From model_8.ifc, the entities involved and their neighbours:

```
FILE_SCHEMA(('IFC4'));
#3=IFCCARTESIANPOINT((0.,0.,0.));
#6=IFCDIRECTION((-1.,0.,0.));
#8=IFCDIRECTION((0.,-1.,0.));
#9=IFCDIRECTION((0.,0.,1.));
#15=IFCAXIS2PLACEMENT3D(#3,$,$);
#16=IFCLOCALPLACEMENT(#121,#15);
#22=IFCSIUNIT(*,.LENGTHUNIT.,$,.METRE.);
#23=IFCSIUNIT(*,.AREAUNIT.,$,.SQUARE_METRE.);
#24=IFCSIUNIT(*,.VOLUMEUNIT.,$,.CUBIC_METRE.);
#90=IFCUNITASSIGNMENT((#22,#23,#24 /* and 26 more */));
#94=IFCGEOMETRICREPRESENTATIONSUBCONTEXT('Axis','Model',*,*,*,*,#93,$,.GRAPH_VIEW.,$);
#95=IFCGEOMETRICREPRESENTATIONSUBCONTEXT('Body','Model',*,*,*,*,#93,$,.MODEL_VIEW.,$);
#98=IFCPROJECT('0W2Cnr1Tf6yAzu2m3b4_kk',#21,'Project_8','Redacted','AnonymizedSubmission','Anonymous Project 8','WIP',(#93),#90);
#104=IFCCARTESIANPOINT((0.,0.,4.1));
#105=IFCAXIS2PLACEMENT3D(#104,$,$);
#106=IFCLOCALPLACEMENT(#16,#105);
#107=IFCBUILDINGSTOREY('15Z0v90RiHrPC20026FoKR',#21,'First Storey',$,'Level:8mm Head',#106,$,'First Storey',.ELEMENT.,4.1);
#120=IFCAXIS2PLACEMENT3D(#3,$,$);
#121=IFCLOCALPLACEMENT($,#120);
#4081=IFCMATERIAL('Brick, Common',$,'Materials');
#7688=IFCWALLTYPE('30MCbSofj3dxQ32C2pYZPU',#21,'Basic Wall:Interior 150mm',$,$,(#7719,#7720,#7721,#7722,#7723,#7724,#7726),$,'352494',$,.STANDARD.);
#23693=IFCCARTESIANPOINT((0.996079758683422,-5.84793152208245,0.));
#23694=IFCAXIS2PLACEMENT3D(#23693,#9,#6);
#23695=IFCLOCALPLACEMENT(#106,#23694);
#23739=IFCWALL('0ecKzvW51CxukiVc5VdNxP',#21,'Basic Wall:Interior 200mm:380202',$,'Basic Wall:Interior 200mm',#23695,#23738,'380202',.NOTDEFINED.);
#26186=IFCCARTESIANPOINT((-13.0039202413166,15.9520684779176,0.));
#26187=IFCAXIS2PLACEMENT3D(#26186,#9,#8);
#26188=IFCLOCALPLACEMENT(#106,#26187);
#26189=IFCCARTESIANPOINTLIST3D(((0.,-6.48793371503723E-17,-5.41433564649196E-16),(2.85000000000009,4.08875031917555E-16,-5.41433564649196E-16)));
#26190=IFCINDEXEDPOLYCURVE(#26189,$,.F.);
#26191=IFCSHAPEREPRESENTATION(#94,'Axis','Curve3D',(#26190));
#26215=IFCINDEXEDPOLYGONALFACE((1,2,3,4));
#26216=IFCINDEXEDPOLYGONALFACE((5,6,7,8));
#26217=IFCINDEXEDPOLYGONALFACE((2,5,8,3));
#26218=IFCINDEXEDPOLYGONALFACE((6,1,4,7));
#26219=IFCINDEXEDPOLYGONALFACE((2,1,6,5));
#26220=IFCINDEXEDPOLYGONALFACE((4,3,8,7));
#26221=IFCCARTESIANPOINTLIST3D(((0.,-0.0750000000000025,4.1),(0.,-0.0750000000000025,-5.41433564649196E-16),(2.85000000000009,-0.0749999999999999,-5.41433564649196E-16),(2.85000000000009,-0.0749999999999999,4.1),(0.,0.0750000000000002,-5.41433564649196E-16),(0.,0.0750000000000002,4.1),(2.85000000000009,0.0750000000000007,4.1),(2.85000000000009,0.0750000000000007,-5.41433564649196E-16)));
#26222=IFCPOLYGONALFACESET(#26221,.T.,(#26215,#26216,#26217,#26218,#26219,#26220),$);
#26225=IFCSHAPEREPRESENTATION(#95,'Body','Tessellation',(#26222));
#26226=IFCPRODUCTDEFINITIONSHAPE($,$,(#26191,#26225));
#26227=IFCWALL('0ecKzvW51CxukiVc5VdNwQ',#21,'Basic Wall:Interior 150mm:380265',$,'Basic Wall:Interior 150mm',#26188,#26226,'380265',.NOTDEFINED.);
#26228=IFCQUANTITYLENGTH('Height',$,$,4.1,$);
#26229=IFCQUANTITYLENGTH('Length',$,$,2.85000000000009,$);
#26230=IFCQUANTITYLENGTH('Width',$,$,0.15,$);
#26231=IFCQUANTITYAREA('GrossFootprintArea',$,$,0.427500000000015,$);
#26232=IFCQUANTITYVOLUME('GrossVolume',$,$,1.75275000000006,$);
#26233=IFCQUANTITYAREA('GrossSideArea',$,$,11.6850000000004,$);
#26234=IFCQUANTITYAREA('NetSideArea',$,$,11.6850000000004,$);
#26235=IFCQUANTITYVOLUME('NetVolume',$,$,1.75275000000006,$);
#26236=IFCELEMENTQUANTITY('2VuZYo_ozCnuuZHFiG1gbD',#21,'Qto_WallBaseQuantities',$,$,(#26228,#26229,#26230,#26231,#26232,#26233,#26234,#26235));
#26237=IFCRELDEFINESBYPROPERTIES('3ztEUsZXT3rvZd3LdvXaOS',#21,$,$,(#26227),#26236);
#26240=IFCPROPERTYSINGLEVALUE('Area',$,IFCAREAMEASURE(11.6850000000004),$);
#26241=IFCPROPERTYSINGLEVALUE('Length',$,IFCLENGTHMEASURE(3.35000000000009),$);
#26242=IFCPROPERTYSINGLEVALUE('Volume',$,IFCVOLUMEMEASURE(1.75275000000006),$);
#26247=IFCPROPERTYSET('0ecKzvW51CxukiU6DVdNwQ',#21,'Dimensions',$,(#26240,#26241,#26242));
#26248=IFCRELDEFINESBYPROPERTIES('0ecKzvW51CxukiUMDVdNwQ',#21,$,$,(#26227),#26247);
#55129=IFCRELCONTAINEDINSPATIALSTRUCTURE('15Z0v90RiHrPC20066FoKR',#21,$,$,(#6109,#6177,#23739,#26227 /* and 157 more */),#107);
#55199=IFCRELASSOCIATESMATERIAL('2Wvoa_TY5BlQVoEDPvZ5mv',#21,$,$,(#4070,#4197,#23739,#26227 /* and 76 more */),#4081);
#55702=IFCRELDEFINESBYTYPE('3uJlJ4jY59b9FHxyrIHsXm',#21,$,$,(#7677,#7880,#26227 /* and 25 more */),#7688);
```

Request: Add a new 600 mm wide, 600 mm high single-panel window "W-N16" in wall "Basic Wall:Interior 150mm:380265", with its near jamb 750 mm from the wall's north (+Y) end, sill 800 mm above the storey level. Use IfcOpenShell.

```python
import numpy as np
import ifcopenshell
import ifcopenshell.api.feature
import ifcopenshell.api.geometry
import ifcopenshell.api.pset
import ifcopenshell.api.root
import ifcopenshell.api.spatial
import ifcopenshell.geom
import ifcopenshell.util.element
import ifcopenshell.util.placement
import ifcopenshell.util.representation
import ifcopenshell.util.shape
import ifcopenshell.util.unit

model = ifcopenshell.open("model_8.ifc")
unit_scale = ifcopenshell.util.unit.calculate_unit_scale(model)
area_scale = ifcopenshell.util.unit.calculate_unit_scale(model, "AREAUNIT")
volume_scale = ifcopenshell.util.unit.calculate_unit_scale(model, "VOLUMEUNIT")
settings = ifcopenshell.geom.settings()


def volume(element):
    """Net volume in cubic metres, openings subtracted."""
    shape = ifcopenshell.geom.create_shape(settings, element)
    return ifcopenshell.util.shape.get_volume(shape.geometry)


wall = model.by_guid("0ecKzvW51CxukiVc5VdNwQ")
storey = ifcopenshell.util.element.get_container(wall, ifc_class="IfcBuildingStorey")
context = ifcopenshell.util.representation.get_context(model, "Model", "Body", "MODEL_VIEW")
before = volume(wall)

width, height, from_end, sill = 0.6, 0.6, 0.75, 0.8  # metres

# The wall runs along its own X axis, and the end named is its -X end.
wall_shape = ifcopenshell.geom.create_shape(settings, wall)
x, y, z = ifcopenshell.util.shape.get_vertices(wall_shape.geometry).T
start = x.min() + from_end
face, thickness = float(y.min()), float(y.max() - y.min())
wall_matrix = ifcopenshell.util.placement.get_local_placement(wall.ObjectPlacement)
level = ifcopenshell.util.placement.get_local_placement(storey.ObjectPlacement)[2, 3]


def in_wall(x, y):
    """Placement at x, y metres in the wall's axes, at sill height."""
    matrix = wall_matrix.copy()
    matrix[:, 3] = wall_matrix @ np.array([x / unit_scale, y / unit_scale, 0.0, 1.0])
    matrix[2, 3] = level + sill / unit_scale
    return matrix


# Opening: a box that overshoots both wall faces by 50 mm.
opening = ifcopenshell.api.root.create_entity(model, ifc_class="IfcOpeningElement", predefined_type="OPENING")
box = ifcopenshell.api.geometry.add_wall_representation(
    model, context=context, length=width, height=height, thickness=thickness + 0.1
)
ifcopenshell.api.geometry.assign_representation(model, product=opening, representation=box)
ifcopenshell.api.geometry.edit_object_placement(model, product=opening, matrix=in_wall(start, face - 0.05), is_si=False)
ifcopenshell.api.feature.add_feature(model, feature=opening, element=wall)

window = ifcopenshell.api.root.create_entity(model, ifc_class="IfcWindow", name="W-N16", predefined_type="WINDOW")
window.OverallWidth, window.OverallHeight = width / unit_scale, height / unit_scale
window.PartitioningType = "SINGLE_PANEL"
body = ifcopenshell.api.geometry.add_window_representation(
    model,
    context=context,
    overall_width=window.OverallWidth,
    overall_height=window.OverallHeight,
    partition_type="SINGLE_PANEL",
)
ifcopenshell.api.geometry.assign_representation(model, product=window, representation=body)
ifcopenshell.api.spatial.assign_container(model, products=[window], relating_structure=storey)
ifcopenshell.api.feature.add_filling(model, opening=opening, element=window)

# Centre the window in the wall's thickness.
ifcopenshell.api.geometry.edit_object_placement(model, product=window, matrix=in_wall(start, face), is_si=False)
window_shape = ifcopenshell.geom.create_shape(settings, window)
depth = ifcopenshell.util.shape.get_vertices(window_shape.geometry)[:, 1]
offset = face + thickness / 2 - (depth.min() + depth.max()) / 2
ifcopenshell.api.geometry.edit_object_placement(model, product=window, matrix=in_wall(start, offset), is_si=False)

after = volume(wall)

# Update the wall's stored quantities.
qto = model.by_id(ifcopenshell.util.element.get_pset(wall, "Qto_WallBaseQuantities", should_inherit=False)["id"])
ifcopenshell.api.pset.edit_qto(model, qto=qto, properties={
    "NetSideArea": after / thickness / area_scale,
    "NetVolume": after / volume_scale,
})
pset = model.by_id(ifcopenshell.util.element.get_pset(wall, "Dimensions", should_inherit=False)["id"])
ifcopenshell.api.pset.edit_pset(model, pset=pset, properties={
    "Area": model.create_entity("IfcAreaMeasure", after / thickness / area_scale),
    "Volume": model.create_entity("IfcVolumeMeasure", after / volume_scale),
})

print(f"wall volume {before:.3f} -> {after:.3f} m3")

model.write("model_8_updated.ifc")
```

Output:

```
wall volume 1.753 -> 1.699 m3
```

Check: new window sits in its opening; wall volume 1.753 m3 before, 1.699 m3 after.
